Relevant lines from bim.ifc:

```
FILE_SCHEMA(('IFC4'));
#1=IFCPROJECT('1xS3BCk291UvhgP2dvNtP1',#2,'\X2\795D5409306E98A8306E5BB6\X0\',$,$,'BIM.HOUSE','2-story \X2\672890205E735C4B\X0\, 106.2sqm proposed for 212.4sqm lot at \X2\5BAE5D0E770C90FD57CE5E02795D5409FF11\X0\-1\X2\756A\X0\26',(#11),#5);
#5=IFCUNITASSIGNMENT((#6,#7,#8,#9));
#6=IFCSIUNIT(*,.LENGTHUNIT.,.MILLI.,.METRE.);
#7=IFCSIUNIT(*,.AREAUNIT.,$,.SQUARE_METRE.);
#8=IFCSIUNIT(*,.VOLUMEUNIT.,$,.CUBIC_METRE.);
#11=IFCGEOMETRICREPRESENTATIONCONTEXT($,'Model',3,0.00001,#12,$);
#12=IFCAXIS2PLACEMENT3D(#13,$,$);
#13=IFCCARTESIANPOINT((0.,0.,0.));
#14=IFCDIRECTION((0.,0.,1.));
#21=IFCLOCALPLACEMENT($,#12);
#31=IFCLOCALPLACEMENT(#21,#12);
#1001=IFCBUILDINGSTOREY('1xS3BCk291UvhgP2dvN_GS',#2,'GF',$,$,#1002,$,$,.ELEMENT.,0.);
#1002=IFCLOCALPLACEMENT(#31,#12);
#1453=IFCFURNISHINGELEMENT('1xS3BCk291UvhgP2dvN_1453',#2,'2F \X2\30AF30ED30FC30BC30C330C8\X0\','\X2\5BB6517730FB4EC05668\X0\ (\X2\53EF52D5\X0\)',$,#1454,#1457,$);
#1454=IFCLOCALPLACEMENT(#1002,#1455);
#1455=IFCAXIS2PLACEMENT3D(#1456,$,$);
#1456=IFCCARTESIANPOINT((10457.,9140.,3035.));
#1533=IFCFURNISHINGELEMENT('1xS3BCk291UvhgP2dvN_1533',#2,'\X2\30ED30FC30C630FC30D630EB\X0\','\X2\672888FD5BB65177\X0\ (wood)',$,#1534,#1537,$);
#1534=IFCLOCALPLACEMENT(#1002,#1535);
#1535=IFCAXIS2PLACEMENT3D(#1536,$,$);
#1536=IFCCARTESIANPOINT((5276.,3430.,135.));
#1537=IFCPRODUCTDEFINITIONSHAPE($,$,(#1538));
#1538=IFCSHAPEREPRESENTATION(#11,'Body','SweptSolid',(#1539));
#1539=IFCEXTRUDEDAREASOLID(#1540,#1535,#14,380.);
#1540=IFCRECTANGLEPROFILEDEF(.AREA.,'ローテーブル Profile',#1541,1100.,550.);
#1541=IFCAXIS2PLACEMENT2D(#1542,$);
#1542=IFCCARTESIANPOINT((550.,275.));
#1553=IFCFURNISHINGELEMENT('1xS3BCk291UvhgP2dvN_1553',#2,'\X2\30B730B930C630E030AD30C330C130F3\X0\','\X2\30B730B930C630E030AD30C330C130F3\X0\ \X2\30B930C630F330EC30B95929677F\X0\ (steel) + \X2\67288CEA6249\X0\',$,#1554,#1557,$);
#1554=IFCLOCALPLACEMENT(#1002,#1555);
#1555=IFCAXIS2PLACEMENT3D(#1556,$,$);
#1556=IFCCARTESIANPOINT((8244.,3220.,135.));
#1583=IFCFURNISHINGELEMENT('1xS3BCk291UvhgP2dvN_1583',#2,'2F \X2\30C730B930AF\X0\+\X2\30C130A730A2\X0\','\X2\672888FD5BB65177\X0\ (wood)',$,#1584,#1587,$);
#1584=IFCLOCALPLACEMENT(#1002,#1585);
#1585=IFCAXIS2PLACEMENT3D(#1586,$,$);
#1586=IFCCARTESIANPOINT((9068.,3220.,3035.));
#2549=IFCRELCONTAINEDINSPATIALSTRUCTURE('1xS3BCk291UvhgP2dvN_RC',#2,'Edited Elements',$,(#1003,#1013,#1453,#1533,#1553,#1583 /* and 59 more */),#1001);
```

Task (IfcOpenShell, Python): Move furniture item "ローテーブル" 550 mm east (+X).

```python
import ifcopenshell
import ifcopenshell.api.geometry
import ifcopenshell.util.placement

model = ifcopenshell.open("bim.ifc")

item = model.by_guid("1xS3BCk291UvhgP2dvN_1533")
matrix = ifcopenshell.util.placement.get_local_placement(item.ObjectPlacement)
matrix[0, 3] += 550.0
ifcopenshell.api.geometry.edit_object_placement(model, product=item, matrix=matrix, is_si=False)

print(ifcopenshell.util.placement.get_local_placement(item.ObjectPlacement).round(3) + 0.0)

model.write("bim_rev.ifc")
```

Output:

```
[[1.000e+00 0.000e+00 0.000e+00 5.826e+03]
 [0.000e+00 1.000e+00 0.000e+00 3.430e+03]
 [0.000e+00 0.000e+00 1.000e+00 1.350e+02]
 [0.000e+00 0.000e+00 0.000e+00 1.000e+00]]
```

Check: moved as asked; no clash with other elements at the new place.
